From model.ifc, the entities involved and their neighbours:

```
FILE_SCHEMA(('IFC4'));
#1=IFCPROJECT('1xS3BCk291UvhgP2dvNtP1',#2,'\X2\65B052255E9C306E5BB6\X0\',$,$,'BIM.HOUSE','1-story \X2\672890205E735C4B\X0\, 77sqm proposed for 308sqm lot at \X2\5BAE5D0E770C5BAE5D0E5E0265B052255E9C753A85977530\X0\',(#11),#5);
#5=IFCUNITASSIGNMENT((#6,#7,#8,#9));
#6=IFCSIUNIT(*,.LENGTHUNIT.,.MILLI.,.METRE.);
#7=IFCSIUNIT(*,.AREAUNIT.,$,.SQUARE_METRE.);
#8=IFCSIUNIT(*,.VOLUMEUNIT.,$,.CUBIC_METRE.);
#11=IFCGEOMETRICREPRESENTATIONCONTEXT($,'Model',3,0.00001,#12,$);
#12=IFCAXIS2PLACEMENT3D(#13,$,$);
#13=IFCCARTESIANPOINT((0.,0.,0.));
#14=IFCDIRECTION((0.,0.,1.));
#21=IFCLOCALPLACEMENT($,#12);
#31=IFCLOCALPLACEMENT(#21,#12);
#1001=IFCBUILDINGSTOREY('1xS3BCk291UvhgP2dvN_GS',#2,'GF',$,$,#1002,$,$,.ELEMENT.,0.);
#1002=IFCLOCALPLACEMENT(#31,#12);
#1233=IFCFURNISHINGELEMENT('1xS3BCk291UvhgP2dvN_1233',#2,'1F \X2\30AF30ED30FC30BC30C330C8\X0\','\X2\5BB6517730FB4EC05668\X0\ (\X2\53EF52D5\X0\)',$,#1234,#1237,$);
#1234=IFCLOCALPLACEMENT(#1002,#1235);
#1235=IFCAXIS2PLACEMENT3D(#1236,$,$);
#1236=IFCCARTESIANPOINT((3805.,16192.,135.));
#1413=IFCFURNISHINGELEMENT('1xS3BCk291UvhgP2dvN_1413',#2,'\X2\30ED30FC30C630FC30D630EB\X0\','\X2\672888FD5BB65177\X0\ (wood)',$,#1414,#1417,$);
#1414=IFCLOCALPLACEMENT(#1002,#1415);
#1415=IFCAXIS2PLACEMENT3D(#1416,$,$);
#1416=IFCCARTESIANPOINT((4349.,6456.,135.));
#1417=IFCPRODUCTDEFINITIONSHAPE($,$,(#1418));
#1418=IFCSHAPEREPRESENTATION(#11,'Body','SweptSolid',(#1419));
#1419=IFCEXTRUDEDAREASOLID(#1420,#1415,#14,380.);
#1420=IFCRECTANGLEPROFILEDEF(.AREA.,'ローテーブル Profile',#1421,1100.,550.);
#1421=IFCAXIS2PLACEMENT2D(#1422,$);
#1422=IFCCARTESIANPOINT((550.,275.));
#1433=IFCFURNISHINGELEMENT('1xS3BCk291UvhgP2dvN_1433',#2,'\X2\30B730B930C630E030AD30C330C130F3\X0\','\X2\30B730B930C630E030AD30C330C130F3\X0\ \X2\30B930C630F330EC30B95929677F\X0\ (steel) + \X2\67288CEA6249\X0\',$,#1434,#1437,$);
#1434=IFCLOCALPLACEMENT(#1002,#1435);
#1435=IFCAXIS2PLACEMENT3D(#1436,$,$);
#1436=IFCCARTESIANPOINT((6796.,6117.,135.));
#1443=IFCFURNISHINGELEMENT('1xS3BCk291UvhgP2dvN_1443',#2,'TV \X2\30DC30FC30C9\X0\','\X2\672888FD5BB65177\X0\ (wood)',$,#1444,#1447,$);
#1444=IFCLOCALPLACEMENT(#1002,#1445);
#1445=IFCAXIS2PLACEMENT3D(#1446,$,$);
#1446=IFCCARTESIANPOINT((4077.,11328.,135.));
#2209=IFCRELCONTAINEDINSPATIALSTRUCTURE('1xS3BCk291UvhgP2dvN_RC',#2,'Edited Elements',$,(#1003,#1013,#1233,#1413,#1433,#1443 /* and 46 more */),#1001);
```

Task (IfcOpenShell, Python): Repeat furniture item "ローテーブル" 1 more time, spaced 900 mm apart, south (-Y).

```python
import numpy as np
import ifcopenshell
import ifcopenshell.api.geometry
import ifcopenshell.api.root
import ifcopenshell.util.element
import ifcopenshell.util.placement

model = ifcopenshell.open("model.ifc")


def reuse_history(source, copy):
    """copy_class also copies each property set's owner history, people and application; keep the originals."""
    for rel in copy.IsDefinedBy:
        if rel.is_a("IfcRelDefinesByProperties") and (history := rel.RelatingPropertyDefinition.OwnerHistory):
            rel.RelatingPropertyDefinition.OwnerHistory = source.OwnerHistory
            ifcopenshell.util.element.remove_deep2(model, history)


source = model.by_id(1413)
base = ifcopenshell.util.placement.get_local_placement(source.ObjectPlacement)
step = np.array([0.0, -1.0, 0.0]) * 900.0

for i in range(1, 2):
    copy = ifcopenshell.api.root.copy_class(model, product=source)
    copy.Representation = ifcopenshell.util.element.copy_deep(
        model, source.Representation, exclude=["IfcGeometricRepresentationContext", "IfcRepresentationMap"]
    )
    reuse_history(source, copy)
    matrix = base.copy()
    matrix[:3, 3] += i * step
    print("added at", matrix[:3, 3].round(3) + 0.0)
    ifcopenshell.api.geometry.edit_object_placement(model, product=copy, matrix=matrix, is_si=False)

model.write("model_rev.ifc")
```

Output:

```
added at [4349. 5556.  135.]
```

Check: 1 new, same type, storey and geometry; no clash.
